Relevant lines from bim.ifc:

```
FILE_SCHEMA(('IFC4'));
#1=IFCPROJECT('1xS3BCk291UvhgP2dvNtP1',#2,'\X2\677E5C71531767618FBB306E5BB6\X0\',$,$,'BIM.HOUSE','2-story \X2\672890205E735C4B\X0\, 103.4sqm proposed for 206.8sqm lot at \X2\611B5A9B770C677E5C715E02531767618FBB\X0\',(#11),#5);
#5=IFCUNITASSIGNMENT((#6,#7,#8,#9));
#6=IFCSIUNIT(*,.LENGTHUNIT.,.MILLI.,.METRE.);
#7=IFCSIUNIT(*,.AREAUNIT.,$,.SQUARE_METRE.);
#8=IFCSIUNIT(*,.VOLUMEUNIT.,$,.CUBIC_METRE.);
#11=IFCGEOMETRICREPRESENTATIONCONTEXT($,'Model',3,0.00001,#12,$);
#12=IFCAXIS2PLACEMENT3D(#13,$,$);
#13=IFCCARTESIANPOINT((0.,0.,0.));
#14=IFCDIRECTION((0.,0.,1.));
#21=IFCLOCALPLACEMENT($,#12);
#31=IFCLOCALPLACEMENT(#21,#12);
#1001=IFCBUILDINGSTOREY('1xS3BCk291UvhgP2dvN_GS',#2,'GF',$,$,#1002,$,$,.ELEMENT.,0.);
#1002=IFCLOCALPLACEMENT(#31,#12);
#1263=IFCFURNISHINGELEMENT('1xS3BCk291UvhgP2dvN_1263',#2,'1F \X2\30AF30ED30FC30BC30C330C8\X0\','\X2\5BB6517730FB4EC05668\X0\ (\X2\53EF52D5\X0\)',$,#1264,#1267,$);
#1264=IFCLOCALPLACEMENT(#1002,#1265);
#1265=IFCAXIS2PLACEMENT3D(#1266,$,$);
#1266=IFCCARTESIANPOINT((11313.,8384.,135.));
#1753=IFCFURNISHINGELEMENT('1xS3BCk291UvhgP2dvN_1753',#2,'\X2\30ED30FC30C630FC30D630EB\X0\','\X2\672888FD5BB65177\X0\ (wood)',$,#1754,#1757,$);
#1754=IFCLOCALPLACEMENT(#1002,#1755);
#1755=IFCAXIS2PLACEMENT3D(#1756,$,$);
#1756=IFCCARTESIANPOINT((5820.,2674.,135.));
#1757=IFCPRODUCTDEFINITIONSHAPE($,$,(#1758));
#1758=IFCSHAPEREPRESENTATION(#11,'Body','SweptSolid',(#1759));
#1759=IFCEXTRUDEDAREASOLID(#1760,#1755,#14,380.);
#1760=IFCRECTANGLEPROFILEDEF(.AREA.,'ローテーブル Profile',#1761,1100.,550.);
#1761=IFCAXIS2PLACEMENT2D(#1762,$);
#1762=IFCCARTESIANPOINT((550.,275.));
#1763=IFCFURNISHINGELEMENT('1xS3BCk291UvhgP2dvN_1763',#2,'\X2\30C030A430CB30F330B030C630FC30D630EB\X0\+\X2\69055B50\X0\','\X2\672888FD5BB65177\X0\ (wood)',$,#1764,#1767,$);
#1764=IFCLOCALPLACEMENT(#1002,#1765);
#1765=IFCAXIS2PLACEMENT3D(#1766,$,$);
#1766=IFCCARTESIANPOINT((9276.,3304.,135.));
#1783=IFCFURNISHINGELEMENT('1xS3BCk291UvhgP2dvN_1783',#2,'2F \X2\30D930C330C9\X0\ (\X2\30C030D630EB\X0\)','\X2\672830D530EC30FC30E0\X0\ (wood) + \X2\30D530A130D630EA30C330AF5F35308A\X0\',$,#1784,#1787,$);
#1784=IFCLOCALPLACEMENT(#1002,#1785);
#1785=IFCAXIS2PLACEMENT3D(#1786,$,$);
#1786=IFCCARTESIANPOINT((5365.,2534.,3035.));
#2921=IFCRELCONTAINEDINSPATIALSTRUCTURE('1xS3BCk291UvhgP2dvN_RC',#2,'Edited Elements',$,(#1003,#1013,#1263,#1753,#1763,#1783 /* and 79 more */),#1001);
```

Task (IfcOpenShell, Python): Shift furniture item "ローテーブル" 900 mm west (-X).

```python
import ifcopenshell
import ifcopenshell.api.geometry
import ifcopenshell.util.placement
import ifcopenshell.util.unit

model = ifcopenshell.open("bim.ifc")
unit_scale = ifcopenshell.util.unit.calculate_unit_scale(model)

item = model.by_guid("1xS3BCk291UvhgP2dvN_1753")
matrix = ifcopenshell.util.placement.get_local_placement(item.ObjectPlacement)
matrix[0, 3] -= 0.9 / unit_scale
ifcopenshell.api.geometry.edit_object_placement(model, product=item, matrix=matrix, is_si=False)

print(ifcopenshell.util.placement.get_local_placement(item.ObjectPlacement).round(3) + 0.0)

model.write("bim_rev.ifc")
```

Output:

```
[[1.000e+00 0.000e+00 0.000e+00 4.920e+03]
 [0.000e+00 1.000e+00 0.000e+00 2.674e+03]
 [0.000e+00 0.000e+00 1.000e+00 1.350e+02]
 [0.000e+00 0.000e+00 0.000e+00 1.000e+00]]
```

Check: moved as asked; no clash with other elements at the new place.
